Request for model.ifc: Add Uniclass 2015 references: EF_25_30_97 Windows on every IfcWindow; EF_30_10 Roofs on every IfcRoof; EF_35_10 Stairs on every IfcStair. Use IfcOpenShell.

First a look at what the model holds.

```python
import ifcopenshell

model = ifcopenshell.open("model.ifc")
print(model.schema)
print("classifications:", [c.Name for c in model.by_type("IfcClassification")])
for ifc_class in ("IfcDoor", "IfcRoof", "IfcStair", "IfcWall", "IfcWindow"):
    print(ifc_class, len(model.by_type(ifc_class)))
```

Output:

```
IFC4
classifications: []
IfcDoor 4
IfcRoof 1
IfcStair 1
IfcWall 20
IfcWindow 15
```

```python
import ifcopenshell
import ifcopenshell.api.classification

model = ifcopenshell.open("model.ifc")

system = ifcopenshell.api.classification.add_classification(model, classification="Uniclass 2015")

codes = {
    "IfcWindow": ("EF_25_30_97", "Windows"),
    "IfcRoof": ("EF_30_10", "Roofs"),
    "IfcStair": ("EF_35_10", "Stairs"),
}
for ifc_class, (code, name) in codes.items():
    products = model.by_type(ifc_class)
    ifcopenshell.api.classification.add_reference(
        model, products=products, classification=system, identification=code, name=name
    )
    print(code, len(products))

model.write("model_v2.ifc")
```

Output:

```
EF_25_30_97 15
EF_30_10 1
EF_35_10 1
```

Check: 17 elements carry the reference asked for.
